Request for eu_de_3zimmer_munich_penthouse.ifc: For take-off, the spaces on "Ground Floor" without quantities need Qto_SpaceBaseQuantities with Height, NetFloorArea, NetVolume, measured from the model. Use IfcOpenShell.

First a look at what the model holds.

```python
import ifcopenshell
import ifcopenshell.util.element
import ifcopenshell.util.unit

model = ifcopenshell.open("eu_de_3zimmer_munich_penthouse.ifc")
print(model.schema)
for unit_type in ("LENGTHUNIT", "AREAUNIT", "VOLUMEUNIT"):
    print(unit_type, ifcopenshell.util.unit.calculate_unit_scale(model, unit_type))
storey = next(s for s in model.by_type("IfcBuildingStorey") if s.Name == "Ground Floor")
spaces = [e for e in ifcopenshell.util.element.get_decomposition(storey) if e.is_a("IfcSpace")]
for e in sorted(spaces, key=lambda e: e.id()):
    print(e.id(), e.is_a(), e.Name, list(ifcopenshell.util.element.get_psets(e, qtos_only=True)), sep=" | ")
```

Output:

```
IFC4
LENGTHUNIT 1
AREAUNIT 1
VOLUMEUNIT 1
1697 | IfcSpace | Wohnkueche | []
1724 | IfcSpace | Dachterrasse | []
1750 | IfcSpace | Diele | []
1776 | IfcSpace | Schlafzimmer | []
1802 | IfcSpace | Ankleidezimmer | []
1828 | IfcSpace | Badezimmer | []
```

```python
import ifcopenshell
import ifcopenshell.api.pset
import ifcopenshell.geom
import ifcopenshell.util.element
import ifcopenshell.util.shape
import ifcopenshell.util.unit

model = ifcopenshell.open("eu_de_3zimmer_munich_penthouse.ifc")
unit_scale = ifcopenshell.util.unit.calculate_unit_scale(model)
area_scale = ifcopenshell.util.unit.calculate_unit_scale(model, "AREAUNIT")
volume_scale = ifcopenshell.util.unit.calculate_unit_scale(model, "VOLUMEUNIT")
settings = ifcopenshell.geom.settings()

storey = next(s for s in model.by_type("IfcBuildingStorey") if s.Name == "Ground Floor")
spaces = [e for e in ifcopenshell.util.element.get_decomposition(storey) if e.is_a("IfcSpace")]

for e in sorted(spaces, key=lambda e: e.id()):
    if ifcopenshell.util.element.get_psets(e, qtos_only=True, should_inherit=False):
        continue
    # Geometry comes back in metres, in the element's own axes.
    shape = ifcopenshell.geom.create_shape(settings, e)
    values = {
        "Height": ifcopenshell.util.shape.get_z(shape.geometry) / unit_scale,
        "NetFloorArea": ifcopenshell.util.shape.get_footprint_area(shape.geometry) / area_scale,
        "NetVolume": ifcopenshell.util.shape.get_volume(shape.geometry) / volume_scale,
    }
    qto = ifcopenshell.api.pset.add_qto(model, product=e, name="Qto_SpaceBaseQuantities")
    ifcopenshell.api.pset.edit_qto(model, qto=qto, properties=values)
    print(e.id(), {k: round(v, 3) for k, v in values.items()})

model.write("eu_de_3zimmer_munich_penthouse_edited.ifc")
```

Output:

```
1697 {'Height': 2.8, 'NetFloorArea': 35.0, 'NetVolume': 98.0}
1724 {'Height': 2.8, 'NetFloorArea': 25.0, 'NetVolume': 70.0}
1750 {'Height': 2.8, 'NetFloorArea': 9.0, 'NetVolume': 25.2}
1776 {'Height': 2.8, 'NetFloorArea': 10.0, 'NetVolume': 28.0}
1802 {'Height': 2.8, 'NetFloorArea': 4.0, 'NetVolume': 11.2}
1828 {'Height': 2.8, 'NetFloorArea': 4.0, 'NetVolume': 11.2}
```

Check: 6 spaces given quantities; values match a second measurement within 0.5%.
